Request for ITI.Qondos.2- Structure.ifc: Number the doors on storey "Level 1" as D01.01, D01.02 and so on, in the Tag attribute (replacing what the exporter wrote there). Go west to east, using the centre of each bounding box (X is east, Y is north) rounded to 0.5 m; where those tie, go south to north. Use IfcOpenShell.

First a look at what the model holds.

```python
import ifcopenshell
import ifcopenshell.util.element
import ifcopenshell.util.placement

model = ifcopenshell.open("ITI.Qondos.2- Structure.ifc")
print(model.schema)
storey = next(s for s in model.by_type("IfcBuildingStorey") if s.Name == "Level 1")
doors = [e for e in ifcopenshell.util.element.get_decomposition(storey) if e.is_a("IfcDoor")]
for e in sorted(doors, key=lambda e: e.id()):
    origin = ifcopenshell.util.placement.get_local_placement(e.ObjectPlacement)[:3, 3]
    print(e.id(), e.Tag, e.Name, origin.round(2) + 0.0, sep=" | ")
```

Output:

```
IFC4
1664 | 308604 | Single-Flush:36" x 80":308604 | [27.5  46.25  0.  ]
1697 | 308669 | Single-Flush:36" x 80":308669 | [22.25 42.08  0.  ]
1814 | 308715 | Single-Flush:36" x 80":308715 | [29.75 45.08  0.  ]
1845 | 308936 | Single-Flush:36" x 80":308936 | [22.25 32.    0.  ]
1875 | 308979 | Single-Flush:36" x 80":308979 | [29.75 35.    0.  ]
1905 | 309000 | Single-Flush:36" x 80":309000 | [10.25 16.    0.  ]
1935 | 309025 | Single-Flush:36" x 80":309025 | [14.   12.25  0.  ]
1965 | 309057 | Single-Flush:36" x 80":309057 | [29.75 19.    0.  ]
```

```python
import ifcopenshell
import ifcopenshell.geom
import ifcopenshell.util.element
import ifcopenshell.util.shape

model = ifcopenshell.open("ITI.Qondos.2- Structure.ifc")
settings = ifcopenshell.geom.settings()
settings.set("use-world-coords", True)


def centre(element):
    shape = ifcopenshell.geom.create_shape(settings, element)
    return ifcopenshell.util.shape.get_bbox_centroid(shape.geometry)


storey = next(s for s in model.by_type("IfcBuildingStorey") if s.Name == "Level 1")
doors = [e for e in ifcopenshell.util.element.get_decomposition(storey) if e.is_a("IfcDoor")]

# Insertion points can sit at a corner or the storey origin, so sort by the geometry (in metres).
centres = {e: centre(e) for e in doors}
doors.sort(key=lambda e: (round(centres[e][0] / 0.5), centres[e][1]))

for i, e in enumerate(doors, start=1):
    number = f"D01.{i:02d}"
    e.Tag = number
    print(e.id(), number)

model.write("ITI.Qondos.2- Structure_updated.ifc")
```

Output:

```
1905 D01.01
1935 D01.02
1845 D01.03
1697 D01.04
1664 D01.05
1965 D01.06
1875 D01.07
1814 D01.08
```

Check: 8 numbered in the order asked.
